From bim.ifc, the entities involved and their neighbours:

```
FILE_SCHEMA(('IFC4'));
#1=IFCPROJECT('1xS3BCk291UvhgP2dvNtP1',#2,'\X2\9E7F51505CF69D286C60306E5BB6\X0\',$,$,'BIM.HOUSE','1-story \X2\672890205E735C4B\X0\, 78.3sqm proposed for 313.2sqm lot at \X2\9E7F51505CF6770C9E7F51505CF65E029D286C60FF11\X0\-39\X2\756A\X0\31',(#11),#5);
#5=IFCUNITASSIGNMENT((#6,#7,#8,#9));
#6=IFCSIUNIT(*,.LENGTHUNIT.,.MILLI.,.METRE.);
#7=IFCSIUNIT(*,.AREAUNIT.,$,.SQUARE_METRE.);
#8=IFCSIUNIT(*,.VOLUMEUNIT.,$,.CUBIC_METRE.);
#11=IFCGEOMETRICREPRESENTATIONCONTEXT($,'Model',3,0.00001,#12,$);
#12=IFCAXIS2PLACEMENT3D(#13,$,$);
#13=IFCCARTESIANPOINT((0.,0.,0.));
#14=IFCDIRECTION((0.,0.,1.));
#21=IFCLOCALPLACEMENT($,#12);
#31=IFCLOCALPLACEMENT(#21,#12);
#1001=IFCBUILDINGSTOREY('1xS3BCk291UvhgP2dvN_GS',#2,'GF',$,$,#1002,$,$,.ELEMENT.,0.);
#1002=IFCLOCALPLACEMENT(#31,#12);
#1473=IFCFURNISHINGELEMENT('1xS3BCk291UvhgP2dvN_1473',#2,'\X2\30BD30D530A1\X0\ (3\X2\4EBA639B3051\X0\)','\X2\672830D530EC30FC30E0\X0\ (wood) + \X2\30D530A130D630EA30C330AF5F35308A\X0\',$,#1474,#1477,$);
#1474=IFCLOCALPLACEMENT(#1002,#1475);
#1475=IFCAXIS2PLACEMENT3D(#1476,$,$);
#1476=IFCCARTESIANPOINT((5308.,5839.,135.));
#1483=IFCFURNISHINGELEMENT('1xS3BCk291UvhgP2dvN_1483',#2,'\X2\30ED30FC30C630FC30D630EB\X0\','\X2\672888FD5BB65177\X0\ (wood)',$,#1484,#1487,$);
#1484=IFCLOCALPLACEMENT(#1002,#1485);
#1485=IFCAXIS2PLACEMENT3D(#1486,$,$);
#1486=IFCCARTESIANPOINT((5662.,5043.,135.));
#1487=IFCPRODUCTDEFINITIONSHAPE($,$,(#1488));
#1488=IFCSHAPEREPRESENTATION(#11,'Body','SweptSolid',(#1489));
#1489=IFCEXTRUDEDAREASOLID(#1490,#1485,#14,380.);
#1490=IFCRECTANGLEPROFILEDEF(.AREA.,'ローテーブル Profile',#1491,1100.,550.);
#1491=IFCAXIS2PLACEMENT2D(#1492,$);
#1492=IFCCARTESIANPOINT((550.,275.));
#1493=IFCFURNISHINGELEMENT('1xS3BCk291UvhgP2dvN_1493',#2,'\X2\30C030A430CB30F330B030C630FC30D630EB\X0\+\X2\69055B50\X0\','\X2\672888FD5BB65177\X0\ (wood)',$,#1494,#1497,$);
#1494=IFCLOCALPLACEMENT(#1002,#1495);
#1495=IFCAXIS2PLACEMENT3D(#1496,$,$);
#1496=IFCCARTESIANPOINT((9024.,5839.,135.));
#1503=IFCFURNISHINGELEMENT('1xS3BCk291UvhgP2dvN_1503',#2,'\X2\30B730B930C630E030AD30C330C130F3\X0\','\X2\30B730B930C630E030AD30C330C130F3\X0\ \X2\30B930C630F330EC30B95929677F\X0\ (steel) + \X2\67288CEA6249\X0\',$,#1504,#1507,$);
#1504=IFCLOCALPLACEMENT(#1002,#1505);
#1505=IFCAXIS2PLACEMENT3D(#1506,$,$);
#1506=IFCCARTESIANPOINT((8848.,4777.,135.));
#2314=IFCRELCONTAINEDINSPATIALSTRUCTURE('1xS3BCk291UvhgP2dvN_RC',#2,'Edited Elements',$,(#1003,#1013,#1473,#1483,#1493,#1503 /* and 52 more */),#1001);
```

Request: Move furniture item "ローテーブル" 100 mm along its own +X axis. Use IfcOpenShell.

```python
import ifcopenshell
import ifcopenshell.api.geometry
import ifcopenshell.util.placement
import ifcopenshell.util.unit

model = ifcopenshell.open("bim.ifc")
unit_scale = ifcopenshell.util.unit.calculate_unit_scale(model)

item = model.by_id(1483)
matrix = ifcopenshell.util.placement.get_local_placement(item.ObjectPlacement)
matrix[:3, 3] += matrix[:3, 0] * 0.1 / unit_scale
ifcopenshell.api.geometry.edit_object_placement(model, product=item, matrix=matrix, is_si=False)

print(ifcopenshell.util.placement.get_local_placement(item.ObjectPlacement).round(3) + 0.0)

model.write("bim-out.ifc")
```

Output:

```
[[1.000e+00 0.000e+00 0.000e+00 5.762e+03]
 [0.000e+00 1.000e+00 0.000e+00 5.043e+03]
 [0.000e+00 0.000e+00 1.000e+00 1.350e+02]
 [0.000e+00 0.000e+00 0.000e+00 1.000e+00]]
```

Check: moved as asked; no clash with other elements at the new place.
